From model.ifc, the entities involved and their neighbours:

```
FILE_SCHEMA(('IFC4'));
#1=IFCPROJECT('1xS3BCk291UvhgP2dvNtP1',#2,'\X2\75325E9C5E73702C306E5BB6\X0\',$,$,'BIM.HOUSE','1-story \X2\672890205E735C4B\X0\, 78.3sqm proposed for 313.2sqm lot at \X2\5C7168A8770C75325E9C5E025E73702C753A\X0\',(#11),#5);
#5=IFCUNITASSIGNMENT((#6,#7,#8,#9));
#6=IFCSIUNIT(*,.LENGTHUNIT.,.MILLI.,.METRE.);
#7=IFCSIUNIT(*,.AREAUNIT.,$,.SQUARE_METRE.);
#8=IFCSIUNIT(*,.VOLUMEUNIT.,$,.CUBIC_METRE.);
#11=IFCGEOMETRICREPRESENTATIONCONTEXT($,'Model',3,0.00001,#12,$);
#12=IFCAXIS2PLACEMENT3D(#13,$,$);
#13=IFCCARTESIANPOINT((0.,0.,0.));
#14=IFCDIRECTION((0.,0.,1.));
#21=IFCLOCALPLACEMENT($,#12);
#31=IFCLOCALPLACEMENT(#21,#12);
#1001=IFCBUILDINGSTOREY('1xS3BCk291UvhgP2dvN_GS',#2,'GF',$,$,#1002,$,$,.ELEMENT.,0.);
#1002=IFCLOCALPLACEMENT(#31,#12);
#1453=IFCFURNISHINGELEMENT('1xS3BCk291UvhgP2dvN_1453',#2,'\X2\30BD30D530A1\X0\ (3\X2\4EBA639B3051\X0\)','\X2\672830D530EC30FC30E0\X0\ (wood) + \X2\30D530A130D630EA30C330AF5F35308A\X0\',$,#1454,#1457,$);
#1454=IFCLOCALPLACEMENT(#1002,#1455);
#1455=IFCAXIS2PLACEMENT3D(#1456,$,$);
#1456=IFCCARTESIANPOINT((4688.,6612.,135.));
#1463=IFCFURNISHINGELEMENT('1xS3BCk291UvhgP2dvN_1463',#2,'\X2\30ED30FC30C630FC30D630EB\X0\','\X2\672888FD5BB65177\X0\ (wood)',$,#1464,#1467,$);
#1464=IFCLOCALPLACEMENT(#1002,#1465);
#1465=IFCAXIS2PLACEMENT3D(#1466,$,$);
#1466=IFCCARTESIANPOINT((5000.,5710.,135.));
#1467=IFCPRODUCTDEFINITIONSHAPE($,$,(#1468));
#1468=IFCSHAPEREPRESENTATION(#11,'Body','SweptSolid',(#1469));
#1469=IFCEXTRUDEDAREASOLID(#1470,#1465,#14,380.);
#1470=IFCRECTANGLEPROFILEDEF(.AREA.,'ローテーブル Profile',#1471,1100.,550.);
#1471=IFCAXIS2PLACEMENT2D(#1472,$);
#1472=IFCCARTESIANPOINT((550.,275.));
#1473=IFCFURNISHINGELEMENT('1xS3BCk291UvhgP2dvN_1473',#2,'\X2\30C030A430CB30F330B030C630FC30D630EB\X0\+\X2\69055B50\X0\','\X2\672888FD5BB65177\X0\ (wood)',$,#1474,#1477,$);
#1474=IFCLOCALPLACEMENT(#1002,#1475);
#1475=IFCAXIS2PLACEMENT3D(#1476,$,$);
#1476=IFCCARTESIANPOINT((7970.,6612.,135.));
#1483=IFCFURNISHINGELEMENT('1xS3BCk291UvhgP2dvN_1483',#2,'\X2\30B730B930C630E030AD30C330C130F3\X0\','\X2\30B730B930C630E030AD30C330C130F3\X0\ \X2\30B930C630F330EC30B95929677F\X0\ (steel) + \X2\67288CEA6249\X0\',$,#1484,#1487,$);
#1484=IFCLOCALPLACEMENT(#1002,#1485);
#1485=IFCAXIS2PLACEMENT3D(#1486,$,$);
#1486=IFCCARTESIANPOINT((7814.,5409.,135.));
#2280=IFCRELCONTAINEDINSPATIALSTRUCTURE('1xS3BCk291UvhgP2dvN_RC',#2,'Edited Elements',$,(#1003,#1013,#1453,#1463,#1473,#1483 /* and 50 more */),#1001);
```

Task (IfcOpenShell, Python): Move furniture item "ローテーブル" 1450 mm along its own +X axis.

```python
import ifcopenshell
import ifcopenshell.api.geometry
import ifcopenshell.util.placement

model = ifcopenshell.open("model.ifc")

item = model.by_guid("1xS3BCk291UvhgP2dvN_1463")
matrix = ifcopenshell.util.placement.get_local_placement(item.ObjectPlacement)
matrix[:3, 3] += matrix[:3, 0] * 1450.0
ifcopenshell.api.geometry.edit_object_placement(model, product=item, matrix=matrix, is_si=False)

print(ifcopenshell.util.placement.get_local_placement(item.ObjectPlacement).round(3) + 0.0)

model.write("model_v2.ifc")
```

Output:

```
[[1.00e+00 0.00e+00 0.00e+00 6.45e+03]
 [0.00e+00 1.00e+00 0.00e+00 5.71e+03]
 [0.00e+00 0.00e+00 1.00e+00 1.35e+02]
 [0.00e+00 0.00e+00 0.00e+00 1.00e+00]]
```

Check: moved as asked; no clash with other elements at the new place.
